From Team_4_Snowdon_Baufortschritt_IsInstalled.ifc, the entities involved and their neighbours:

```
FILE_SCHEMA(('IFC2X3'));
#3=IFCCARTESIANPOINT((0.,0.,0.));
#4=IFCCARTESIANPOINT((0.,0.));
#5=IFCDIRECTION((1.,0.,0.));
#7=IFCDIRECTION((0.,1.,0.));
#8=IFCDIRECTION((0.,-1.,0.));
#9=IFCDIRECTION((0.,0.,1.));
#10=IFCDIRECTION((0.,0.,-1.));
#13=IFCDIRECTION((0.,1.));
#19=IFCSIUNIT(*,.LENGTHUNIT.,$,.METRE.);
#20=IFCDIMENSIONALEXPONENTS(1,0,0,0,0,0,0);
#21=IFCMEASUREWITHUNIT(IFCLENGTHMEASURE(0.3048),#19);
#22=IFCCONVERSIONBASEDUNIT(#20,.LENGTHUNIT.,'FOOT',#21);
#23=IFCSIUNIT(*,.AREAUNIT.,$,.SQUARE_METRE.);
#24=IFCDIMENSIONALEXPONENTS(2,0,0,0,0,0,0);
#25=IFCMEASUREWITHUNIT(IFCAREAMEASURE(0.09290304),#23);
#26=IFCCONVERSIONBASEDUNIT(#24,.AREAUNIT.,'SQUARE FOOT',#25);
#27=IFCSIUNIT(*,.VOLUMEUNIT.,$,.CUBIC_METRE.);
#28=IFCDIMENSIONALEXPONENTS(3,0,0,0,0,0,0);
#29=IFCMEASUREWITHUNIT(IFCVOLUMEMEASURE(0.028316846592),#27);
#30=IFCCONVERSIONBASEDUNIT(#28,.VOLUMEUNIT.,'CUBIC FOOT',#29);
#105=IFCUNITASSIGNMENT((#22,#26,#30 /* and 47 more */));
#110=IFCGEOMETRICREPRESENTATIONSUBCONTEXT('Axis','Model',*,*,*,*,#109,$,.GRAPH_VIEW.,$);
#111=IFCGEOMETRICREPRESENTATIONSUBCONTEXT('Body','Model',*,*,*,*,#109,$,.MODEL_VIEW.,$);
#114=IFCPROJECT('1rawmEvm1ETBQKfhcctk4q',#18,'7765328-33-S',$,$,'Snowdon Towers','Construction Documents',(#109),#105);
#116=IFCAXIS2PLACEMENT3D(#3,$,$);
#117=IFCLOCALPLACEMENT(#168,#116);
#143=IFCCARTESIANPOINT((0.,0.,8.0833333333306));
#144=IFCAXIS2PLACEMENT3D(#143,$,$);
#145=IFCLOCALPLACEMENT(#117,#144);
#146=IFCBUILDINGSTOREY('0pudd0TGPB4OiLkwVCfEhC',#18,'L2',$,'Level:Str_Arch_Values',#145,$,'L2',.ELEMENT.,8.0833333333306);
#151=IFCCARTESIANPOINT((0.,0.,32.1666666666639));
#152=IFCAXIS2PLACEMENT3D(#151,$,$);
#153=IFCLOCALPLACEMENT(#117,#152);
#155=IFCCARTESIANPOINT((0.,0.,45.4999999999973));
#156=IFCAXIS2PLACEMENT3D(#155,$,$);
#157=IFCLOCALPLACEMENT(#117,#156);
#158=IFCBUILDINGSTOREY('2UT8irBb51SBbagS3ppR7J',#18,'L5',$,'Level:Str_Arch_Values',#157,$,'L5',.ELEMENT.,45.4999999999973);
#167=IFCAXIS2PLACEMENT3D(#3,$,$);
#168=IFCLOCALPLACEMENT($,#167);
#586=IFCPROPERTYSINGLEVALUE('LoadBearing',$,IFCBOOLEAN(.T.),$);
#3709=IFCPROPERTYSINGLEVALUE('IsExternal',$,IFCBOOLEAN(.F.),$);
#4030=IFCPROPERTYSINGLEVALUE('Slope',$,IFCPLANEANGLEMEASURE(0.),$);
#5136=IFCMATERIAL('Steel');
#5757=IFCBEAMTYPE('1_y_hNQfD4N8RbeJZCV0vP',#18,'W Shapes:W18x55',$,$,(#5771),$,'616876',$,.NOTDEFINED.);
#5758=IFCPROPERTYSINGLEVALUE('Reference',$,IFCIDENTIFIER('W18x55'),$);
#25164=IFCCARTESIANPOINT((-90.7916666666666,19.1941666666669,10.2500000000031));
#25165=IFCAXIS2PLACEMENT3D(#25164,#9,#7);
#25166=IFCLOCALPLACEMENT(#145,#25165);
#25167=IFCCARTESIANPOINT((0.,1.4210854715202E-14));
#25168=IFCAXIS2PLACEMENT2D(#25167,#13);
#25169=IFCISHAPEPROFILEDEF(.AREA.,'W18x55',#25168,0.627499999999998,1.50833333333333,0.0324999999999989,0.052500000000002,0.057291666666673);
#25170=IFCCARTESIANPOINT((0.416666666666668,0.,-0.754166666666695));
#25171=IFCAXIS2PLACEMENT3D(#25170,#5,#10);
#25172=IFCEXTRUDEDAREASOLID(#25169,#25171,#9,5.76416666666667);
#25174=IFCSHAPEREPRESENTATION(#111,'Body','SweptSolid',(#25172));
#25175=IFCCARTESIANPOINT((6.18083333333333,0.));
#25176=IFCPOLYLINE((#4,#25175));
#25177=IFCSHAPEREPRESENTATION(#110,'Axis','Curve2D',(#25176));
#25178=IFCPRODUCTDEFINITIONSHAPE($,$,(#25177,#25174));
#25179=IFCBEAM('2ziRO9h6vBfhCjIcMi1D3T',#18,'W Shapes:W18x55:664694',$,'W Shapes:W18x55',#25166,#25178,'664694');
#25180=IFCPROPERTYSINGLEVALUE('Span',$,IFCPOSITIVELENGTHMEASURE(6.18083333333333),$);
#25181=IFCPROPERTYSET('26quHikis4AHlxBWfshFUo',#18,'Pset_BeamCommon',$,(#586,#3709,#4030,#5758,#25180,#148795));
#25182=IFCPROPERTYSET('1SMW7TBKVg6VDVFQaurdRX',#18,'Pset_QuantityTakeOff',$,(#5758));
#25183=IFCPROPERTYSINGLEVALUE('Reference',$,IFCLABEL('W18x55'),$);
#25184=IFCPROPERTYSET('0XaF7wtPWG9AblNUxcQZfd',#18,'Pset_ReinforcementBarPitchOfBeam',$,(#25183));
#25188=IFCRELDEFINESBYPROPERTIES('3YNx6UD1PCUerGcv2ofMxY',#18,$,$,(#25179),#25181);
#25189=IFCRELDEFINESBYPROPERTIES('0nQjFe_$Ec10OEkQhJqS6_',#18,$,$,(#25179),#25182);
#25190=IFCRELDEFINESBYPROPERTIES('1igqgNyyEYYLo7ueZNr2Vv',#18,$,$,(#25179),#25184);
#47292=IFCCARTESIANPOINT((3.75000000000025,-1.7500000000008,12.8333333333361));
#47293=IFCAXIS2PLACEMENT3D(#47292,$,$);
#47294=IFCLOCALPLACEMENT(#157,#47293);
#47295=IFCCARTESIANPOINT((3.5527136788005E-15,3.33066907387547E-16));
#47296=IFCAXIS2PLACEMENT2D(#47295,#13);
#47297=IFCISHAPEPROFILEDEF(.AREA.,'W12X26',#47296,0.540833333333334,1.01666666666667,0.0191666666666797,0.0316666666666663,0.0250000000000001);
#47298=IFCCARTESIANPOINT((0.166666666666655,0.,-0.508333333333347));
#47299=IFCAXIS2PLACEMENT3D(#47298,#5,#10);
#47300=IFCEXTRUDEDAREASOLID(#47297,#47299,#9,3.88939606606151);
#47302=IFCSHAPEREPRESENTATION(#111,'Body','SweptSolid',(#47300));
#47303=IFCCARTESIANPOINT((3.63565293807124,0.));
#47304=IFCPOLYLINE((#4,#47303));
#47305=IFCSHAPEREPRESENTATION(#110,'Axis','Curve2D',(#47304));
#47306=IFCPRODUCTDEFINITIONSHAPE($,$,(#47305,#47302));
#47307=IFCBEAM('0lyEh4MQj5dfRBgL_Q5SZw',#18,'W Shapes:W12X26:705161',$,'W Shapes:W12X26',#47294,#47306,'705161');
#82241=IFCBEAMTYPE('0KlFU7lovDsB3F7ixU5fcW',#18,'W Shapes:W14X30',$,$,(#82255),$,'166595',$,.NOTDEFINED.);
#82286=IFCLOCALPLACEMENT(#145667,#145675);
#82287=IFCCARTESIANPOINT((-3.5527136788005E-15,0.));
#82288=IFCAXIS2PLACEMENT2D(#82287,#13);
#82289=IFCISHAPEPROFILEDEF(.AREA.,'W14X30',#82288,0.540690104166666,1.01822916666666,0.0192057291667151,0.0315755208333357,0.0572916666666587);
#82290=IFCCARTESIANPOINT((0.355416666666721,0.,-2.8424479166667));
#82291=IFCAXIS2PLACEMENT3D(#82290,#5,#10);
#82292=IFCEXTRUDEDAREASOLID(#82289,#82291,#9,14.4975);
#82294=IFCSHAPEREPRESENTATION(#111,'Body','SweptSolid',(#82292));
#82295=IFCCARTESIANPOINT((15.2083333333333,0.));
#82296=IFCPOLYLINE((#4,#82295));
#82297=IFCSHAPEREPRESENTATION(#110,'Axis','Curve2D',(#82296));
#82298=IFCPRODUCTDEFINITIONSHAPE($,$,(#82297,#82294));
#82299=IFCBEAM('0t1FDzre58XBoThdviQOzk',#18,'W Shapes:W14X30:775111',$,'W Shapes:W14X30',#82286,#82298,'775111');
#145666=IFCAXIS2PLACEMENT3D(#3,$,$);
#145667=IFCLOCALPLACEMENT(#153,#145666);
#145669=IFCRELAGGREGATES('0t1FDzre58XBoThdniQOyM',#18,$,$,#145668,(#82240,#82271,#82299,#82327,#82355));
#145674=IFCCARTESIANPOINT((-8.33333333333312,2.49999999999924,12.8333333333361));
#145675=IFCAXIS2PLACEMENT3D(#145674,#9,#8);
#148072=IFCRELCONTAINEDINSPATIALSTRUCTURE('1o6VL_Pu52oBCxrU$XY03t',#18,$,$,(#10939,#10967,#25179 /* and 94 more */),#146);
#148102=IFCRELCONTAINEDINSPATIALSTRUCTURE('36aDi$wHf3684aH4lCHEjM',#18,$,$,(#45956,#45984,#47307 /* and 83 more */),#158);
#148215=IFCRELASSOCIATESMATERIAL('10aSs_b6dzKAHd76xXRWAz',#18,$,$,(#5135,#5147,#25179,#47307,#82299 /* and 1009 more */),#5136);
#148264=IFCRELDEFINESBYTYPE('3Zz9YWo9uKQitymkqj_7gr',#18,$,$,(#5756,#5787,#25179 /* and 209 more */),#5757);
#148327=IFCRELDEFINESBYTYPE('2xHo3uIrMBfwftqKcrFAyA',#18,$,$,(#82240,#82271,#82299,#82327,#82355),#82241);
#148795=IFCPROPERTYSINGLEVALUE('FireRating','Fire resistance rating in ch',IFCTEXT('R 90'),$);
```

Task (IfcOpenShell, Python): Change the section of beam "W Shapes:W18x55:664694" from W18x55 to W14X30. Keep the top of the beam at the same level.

```python
import ifcopenshell
import ifcopenshell.api.pset
import ifcopenshell.api.type
import ifcopenshell.util.element
import ifcopenshell.util.representation

model = ifcopenshell.open("Team_4_Snowdon_Baufortschritt_IsInstalled.ifc")

member = model.by_id(25179)
source = next(p for p in model.by_type("IfcIShapeProfileDef") if p.ProfileName == "W14X30")

body = ifcopenshell.util.representation.get_representation(member, "Model", "Body")
solid = body.Items[0]
old_profile = solid.SweptArea

# Copy the section's sizes but keep this member's own profile position.
profile = ifcopenshell.util.element.copy(model, source)
# Profiles are centred, so shift by half the change in depth to hold the top.
shift = (old_profile.OverallDepth - profile.OverallDepth) / 2
x, y = old_profile.Position.Location.Coordinates
up = (-1.0, 0.0)  # upwards, in the solid's own plane
location = model.createIfcCartesianPoint((x + up[0] * shift, y + up[1] * shift))
profile.Position = model.createIfcAxis2Placement2D(location, old_profile.Position.RefDirection)
solid.SweptArea = profile
if not model.get_total_inverses(old_profile):
    ifcopenshell.util.element.remove_deep2(model, old_profile)

new_type = model.by_id(82241)
ifcopenshell.api.type.assign_type(
    model, related_objects=[member], relating_type=new_type, should_map_representations=False
)
member.Name = member.Name.replace("W18x55", "W14X30")
member.ObjectType = "W Shapes:W14X30"
pset = model.by_id(ifcopenshell.util.element.get_pset(member, "Pset_BeamCommon", should_inherit=False)["id"])
ifcopenshell.api.pset.edit_pset(model, pset=pset, properties={"Reference": "W14X30"})
pset = model.by_id(ifcopenshell.util.element.get_pset(member, "Pset_QuantityTakeOff", should_inherit=False)["id"])
ifcopenshell.api.pset.edit_pset(model, pset=pset, properties={"Reference": "W14X30"})
pset = model.by_id(ifcopenshell.util.element.get_pset(member, "Pset_ReinforcementBarPitchOfBeam", should_inherit=False)["id"])
ifcopenshell.api.pset.edit_pset(model, pset=pset, properties={"Reference": "W14X30"})

print(solid.SweptArea)

model.write("Team_4_Snowdon_Baufortschritt_IsInstalled-out.ifc")
```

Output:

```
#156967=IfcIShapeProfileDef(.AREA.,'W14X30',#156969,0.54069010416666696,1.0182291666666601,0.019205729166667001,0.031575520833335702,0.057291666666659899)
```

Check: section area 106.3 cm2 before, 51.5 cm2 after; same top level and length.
